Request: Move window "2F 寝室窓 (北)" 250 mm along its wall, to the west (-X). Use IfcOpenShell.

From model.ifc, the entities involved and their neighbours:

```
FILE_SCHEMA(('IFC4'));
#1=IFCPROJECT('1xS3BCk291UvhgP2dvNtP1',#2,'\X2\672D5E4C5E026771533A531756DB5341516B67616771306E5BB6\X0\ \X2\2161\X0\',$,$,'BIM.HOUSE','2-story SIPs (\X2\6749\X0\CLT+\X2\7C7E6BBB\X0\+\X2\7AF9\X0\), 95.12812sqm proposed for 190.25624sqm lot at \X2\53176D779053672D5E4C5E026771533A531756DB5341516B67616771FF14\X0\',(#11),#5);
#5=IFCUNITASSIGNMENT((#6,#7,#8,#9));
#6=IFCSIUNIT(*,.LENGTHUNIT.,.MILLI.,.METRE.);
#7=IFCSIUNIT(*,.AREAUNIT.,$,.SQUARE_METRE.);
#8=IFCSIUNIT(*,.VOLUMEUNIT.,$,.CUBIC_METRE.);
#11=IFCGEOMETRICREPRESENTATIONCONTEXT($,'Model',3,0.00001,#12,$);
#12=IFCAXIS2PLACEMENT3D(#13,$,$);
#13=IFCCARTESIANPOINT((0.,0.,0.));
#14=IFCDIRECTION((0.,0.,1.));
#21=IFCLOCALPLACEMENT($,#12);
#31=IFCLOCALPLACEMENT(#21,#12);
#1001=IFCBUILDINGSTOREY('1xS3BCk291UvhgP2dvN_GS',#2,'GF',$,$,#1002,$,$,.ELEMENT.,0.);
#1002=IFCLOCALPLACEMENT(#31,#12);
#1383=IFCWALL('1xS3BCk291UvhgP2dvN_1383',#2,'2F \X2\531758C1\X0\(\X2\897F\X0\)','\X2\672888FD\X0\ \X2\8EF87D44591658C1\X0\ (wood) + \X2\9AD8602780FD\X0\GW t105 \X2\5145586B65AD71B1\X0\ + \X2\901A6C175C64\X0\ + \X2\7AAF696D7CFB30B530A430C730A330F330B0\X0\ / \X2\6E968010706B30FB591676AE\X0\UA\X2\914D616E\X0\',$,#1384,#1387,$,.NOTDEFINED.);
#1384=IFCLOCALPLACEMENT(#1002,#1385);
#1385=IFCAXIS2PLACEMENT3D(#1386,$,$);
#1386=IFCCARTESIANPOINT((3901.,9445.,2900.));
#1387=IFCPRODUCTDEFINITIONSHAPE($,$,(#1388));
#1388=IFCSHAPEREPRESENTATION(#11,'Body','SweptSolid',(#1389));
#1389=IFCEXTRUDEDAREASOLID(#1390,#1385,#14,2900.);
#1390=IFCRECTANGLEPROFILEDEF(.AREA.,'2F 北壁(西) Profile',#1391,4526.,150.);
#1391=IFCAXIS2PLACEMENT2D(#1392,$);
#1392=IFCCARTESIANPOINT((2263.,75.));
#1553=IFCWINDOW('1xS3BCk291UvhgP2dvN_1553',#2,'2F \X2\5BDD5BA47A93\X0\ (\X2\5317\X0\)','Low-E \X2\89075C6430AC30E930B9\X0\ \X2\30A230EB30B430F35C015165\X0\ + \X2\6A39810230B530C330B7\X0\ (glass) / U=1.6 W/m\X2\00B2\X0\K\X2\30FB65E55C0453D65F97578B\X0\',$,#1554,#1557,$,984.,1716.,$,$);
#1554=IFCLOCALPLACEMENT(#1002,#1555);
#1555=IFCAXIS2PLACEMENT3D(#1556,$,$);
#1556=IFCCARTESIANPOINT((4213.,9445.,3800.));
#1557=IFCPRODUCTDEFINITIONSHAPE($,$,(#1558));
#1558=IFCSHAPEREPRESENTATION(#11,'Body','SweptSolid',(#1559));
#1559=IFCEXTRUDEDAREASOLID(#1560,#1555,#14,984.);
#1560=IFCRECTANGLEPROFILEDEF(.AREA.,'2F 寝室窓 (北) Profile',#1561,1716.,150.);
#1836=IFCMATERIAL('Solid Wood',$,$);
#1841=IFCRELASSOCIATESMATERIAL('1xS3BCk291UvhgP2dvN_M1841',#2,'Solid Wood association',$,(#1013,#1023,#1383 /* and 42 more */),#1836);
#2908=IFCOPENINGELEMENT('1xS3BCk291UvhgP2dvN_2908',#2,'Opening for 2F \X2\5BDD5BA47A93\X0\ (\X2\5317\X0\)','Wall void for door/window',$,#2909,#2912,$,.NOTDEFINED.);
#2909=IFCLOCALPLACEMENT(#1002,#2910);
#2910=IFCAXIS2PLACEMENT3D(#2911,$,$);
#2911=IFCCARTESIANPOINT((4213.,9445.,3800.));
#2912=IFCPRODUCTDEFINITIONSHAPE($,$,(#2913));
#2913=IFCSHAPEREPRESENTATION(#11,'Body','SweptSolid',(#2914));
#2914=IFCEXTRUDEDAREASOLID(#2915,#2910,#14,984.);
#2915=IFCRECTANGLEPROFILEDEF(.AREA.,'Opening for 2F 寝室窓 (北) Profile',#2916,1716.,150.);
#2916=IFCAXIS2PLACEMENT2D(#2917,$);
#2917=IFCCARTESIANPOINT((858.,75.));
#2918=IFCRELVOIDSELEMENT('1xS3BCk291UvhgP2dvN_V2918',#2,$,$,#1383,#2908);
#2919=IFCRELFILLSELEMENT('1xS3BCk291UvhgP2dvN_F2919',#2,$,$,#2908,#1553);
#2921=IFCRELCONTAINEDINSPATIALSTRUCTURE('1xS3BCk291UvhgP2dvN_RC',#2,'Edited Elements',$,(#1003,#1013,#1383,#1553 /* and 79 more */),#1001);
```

```python
import ifcopenshell
import ifcopenshell.api.geometry
import ifcopenshell.util.placement
import ifcopenshell.util.unit

model = ifcopenshell.open("model.ifc")
unit_scale = ifcopenshell.util.unit.calculate_unit_scale(model)

window = model.by_guid("1xS3BCk291UvhgP2dvN_1553")
opening = window.FillsVoids[0].RelatingOpeningElement
wall = opening.VoidsElements[0].RelatingBuildingElement

wall_matrix = ifcopenshell.util.placement.get_local_placement(wall.ObjectPlacement)
shift = wall_matrix[:3, 0] * -0.25 / unit_scale
before = ifcopenshell.util.placement.get_local_placement(window.ObjectPlacement)[:3, 3].copy()

# The window is not placed relative to its opening, so move both.
for product in (opening, window):
    matrix = ifcopenshell.util.placement.get_local_placement(product.ObjectPlacement)
    matrix[:3, 3] += shift
    ifcopenshell.api.geometry.edit_object_placement(model, product=product, matrix=matrix, is_si=False)

after = ifcopenshell.util.placement.get_local_placement(window.ObjectPlacement)[:3, 3]
print("window moved by", (after - before).round(3) + 0.0)

model.write("model_edited.ifc")
```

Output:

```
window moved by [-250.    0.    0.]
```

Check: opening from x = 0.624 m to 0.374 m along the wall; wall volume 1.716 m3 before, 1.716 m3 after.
